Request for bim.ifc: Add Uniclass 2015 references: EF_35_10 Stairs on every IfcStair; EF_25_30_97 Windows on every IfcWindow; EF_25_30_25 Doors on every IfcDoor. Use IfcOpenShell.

First a look at what the model holds.

```python
import ifcopenshell

model = ifcopenshell.open("bim.ifc")
print(model.schema)
print("classifications:", [c.Name for c in model.by_type("IfcClassification")])
for ifc_class in ("IfcDoor", "IfcRoof", "IfcStair", "IfcWall", "IfcWindow"):
    print(ifc_class, len(model.by_type(ifc_class)))
```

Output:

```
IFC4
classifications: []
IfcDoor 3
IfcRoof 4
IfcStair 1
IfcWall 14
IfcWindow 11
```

```python
import ifcopenshell
import ifcopenshell.api.classification

model = ifcopenshell.open("bim.ifc")

system = ifcopenshell.api.classification.add_classification(model, classification="Uniclass 2015")

codes = {
    "IfcStair": ("EF_35_10", "Stairs"),
    "IfcWindow": ("EF_25_30_97", "Windows"),
    "IfcDoor": ("EF_25_30_25", "Doors"),
}
for ifc_class, (code, name) in codes.items():
    products = model.by_type(ifc_class)
    ifcopenshell.api.classification.add_reference(
        model, products=products, classification=system, identification=code, name=name
    )
    print(code, len(products))

model.write("bim_rev.ifc")
```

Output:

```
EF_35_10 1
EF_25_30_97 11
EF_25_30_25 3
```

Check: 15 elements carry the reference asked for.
